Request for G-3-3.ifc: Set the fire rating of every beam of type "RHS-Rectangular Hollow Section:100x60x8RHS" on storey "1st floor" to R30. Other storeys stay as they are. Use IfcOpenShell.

First a look at what the model holds.

```python
import ifcopenshell
import ifcopenshell.util.element

model = ifcopenshell.open("G-3-3.ifc")
print(model.schema)
storey = next(s for s in model.by_type("IfcBuildingStorey") if s.Name == "1st floor")
beams = [e for e in ifcopenshell.util.element.get_decomposition(storey) if e.is_a("IfcBeam")]
seen = {}
for e in beams:
    element_type = ifcopenshell.util.element.get_type(e)
    key = (element_type.Name if element_type != e and element_type else None, ifcopenshell.util.element.get_pset(e, "Pset_BeamCommon", "FireRating"))
    seen[key] = seen.get(key, 0) + 1
for (name, value), count in sorted(seen.items(), key=str):
    print(count, "x", name, "|", value)
```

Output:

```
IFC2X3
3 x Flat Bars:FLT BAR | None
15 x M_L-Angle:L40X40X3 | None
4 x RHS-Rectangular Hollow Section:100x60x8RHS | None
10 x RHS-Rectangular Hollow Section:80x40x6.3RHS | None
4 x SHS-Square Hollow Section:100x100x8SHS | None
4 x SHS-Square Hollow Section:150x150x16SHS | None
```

```python
import ifcopenshell
import ifcopenshell.api.pset
import ifcopenshell.util.element

model = ifcopenshell.open("G-3-3.ifc")

storey = next(s for s in model.by_type("IfcBuildingStorey") if s.Name == "1st floor")
beams = [e for e in ifcopenshell.util.element.get_decomposition(storey) if e.is_a("IfcBeam")]

count = 0
for e in beams:
    element_type = ifcopenshell.util.element.get_type(e)
    if element_type in (None, e) or element_type.Name != "RHS-Rectangular Hollow Section:100x60x8RHS":
        continue
    # add_pset returns the element's existing set when there is one.
    pset = ifcopenshell.api.pset.add_pset(model, product=e, name="Pset_BeamCommon")
    ifcopenshell.api.pset.edit_pset(model, pset=pset, properties={"FireRating": "R30"})
    count += 1

print(count, "beams updated")

model.write("G-3-3_rev.ifc")
```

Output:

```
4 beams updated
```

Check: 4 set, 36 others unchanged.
